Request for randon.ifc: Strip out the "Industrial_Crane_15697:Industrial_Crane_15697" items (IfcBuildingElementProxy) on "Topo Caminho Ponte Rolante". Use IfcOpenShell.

First a look at what the model holds.

```python
import ifcopenshell
import ifcopenshell.util.element

model = ifcopenshell.open("randon.ifc")
print(model.schema)
storey = next(s for s in model.by_type("IfcBuildingStorey") if s.Name == "Topo Caminho Ponte Rolante")
proxies = [e for e in ifcopenshell.util.element.get_decomposition(storey) if e.is_a("IfcBuildingElementProxy")]
seen = {}
for e in proxies:
    element_type = ifcopenshell.util.element.get_type(e)
    name = element_type.Name if element_type not in (None, e) else None
    seen[name] = seen.get(name, 0) + 1
for name, count in sorted(seen.items(), key=str):
    print(count, "x", name)
```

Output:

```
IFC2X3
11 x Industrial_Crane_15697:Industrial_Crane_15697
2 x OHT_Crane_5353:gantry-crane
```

```python
import ifcopenshell
import ifcopenshell.api.root
import ifcopenshell.util.element

model = ifcopenshell.open("randon.ifc")

storey = next(s for s in model.by_type("IfcBuildingStorey") if s.Name == "Topo Caminho Ponte Rolante")
proxies = [e for e in ifcopenshell.util.element.get_decomposition(storey) if e.is_a("IfcBuildingElementProxy")]
targets = [e for e in proxies if (t := ifcopenshell.util.element.get_type(e)) not in (None, e) and t.Name == "Industrial_Crane_15697:Industrial_Crane_15697"]

for e in targets:
    ifcopenshell.api.root.remove_product(model, product=e)
print(len(targets), "removed")

model.write("randon_updated.ifc")
```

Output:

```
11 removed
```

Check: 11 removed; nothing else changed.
